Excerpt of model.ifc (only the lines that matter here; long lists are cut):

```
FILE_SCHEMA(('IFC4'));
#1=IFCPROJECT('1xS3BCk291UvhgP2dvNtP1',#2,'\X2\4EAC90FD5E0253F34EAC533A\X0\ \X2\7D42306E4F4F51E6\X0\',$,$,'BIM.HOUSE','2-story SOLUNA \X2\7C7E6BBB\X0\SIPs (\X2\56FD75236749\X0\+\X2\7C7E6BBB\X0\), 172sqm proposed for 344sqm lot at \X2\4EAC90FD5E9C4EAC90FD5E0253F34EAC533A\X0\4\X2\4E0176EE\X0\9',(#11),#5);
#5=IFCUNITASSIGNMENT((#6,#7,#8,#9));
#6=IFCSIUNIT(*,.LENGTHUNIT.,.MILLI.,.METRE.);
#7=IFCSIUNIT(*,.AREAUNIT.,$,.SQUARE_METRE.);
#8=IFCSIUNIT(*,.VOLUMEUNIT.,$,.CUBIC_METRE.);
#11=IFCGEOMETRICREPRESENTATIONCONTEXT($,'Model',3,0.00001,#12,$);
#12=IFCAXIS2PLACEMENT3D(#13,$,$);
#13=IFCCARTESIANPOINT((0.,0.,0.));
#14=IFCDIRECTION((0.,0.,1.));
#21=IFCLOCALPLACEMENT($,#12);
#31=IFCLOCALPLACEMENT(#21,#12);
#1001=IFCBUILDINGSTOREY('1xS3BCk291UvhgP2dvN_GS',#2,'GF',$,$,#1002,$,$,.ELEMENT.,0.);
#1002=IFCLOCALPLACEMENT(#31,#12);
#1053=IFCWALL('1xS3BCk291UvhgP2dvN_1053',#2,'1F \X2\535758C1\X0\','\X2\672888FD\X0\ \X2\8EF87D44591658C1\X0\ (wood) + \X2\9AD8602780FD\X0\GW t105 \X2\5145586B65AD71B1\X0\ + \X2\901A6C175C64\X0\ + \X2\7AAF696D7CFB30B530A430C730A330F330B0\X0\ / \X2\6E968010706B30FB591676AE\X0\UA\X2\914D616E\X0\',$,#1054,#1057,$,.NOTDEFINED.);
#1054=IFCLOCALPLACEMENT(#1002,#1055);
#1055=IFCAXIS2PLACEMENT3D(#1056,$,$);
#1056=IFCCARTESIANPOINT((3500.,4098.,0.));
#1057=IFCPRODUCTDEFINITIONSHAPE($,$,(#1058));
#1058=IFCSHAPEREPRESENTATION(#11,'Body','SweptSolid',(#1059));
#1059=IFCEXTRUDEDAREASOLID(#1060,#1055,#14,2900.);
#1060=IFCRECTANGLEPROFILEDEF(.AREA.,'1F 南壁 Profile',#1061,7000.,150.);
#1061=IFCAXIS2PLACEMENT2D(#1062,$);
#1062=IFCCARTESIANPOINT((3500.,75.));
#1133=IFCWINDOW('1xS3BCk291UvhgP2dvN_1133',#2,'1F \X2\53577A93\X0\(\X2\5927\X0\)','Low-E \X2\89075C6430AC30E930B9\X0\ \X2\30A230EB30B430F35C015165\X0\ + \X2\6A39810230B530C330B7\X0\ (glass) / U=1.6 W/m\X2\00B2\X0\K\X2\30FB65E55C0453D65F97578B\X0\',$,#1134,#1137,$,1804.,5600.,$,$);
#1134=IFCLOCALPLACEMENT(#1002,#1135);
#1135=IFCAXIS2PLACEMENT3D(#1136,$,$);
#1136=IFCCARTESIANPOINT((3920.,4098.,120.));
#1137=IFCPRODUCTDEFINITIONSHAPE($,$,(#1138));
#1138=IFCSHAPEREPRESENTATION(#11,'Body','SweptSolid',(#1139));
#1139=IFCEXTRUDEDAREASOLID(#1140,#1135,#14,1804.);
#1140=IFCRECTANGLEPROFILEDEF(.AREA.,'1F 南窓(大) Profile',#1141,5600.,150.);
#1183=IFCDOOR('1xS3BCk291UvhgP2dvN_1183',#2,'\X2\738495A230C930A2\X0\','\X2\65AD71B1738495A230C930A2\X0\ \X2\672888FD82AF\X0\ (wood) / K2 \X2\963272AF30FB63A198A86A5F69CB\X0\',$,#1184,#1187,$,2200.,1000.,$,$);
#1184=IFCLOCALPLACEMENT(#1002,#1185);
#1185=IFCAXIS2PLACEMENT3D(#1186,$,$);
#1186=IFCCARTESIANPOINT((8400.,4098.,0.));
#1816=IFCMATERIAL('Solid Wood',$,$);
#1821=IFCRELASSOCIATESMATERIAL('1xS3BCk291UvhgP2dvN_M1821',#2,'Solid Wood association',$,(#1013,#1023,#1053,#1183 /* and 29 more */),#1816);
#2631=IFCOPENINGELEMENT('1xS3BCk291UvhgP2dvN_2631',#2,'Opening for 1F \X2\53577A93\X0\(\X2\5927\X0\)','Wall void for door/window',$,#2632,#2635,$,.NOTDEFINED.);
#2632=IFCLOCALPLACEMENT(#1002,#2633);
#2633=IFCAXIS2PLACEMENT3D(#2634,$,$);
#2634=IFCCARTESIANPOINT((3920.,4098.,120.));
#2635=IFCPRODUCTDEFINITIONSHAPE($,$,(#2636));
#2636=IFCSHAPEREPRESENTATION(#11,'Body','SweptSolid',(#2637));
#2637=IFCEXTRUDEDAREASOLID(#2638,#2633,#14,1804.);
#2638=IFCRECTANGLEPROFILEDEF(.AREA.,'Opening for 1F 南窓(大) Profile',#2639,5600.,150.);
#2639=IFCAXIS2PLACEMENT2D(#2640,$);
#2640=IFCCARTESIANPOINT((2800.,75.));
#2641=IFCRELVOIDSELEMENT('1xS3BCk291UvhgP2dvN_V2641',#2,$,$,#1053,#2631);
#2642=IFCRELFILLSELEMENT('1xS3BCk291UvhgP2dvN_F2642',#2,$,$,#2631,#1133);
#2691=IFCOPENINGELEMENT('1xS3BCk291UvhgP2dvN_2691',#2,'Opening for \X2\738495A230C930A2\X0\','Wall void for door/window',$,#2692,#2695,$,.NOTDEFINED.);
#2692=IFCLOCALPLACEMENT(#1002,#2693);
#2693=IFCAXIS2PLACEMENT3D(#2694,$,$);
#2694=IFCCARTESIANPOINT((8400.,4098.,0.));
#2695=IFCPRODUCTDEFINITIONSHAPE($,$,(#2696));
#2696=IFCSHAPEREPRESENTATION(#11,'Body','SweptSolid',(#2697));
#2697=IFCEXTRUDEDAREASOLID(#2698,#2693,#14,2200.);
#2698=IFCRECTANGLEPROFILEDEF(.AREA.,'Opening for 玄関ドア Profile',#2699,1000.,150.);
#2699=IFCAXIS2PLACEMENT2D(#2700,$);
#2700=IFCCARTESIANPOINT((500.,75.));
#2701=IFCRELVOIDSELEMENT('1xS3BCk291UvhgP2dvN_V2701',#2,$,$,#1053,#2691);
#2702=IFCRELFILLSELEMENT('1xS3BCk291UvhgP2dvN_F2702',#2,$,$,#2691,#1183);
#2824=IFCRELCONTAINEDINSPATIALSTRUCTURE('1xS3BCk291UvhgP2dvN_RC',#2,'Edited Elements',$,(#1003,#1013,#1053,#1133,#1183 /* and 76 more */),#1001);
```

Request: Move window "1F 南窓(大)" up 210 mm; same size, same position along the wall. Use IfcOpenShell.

```python
import numpy as np
import ifcopenshell
import ifcopenshell.api.geometry
import ifcopenshell.util.placement
import ifcopenshell.util.unit

model = ifcopenshell.open("model.ifc")
unit_scale = ifcopenshell.util.unit.calculate_unit_scale(model)

window = model.by_guid("1xS3BCk291UvhgP2dvN_1133")
opening = window.FillsVoids[0].RelatingOpeningElement
dz = 0.21 / unit_scale

shift = np.array([0.0, 0.0, dz])
# The window is not placed relative to its opening, so move both.
for product in (opening, window):
    matrix = ifcopenshell.util.placement.get_local_placement(product.ObjectPlacement)
    matrix[:3, 3] += shift
    ifcopenshell.api.geometry.edit_object_placement(model, product=product, matrix=matrix, is_si=False)

print(f"moved by {dz * unit_scale:+.3f} m")

model.write("model-out.ifc")
```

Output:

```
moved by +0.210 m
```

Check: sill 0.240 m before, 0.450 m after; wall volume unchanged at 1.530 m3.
